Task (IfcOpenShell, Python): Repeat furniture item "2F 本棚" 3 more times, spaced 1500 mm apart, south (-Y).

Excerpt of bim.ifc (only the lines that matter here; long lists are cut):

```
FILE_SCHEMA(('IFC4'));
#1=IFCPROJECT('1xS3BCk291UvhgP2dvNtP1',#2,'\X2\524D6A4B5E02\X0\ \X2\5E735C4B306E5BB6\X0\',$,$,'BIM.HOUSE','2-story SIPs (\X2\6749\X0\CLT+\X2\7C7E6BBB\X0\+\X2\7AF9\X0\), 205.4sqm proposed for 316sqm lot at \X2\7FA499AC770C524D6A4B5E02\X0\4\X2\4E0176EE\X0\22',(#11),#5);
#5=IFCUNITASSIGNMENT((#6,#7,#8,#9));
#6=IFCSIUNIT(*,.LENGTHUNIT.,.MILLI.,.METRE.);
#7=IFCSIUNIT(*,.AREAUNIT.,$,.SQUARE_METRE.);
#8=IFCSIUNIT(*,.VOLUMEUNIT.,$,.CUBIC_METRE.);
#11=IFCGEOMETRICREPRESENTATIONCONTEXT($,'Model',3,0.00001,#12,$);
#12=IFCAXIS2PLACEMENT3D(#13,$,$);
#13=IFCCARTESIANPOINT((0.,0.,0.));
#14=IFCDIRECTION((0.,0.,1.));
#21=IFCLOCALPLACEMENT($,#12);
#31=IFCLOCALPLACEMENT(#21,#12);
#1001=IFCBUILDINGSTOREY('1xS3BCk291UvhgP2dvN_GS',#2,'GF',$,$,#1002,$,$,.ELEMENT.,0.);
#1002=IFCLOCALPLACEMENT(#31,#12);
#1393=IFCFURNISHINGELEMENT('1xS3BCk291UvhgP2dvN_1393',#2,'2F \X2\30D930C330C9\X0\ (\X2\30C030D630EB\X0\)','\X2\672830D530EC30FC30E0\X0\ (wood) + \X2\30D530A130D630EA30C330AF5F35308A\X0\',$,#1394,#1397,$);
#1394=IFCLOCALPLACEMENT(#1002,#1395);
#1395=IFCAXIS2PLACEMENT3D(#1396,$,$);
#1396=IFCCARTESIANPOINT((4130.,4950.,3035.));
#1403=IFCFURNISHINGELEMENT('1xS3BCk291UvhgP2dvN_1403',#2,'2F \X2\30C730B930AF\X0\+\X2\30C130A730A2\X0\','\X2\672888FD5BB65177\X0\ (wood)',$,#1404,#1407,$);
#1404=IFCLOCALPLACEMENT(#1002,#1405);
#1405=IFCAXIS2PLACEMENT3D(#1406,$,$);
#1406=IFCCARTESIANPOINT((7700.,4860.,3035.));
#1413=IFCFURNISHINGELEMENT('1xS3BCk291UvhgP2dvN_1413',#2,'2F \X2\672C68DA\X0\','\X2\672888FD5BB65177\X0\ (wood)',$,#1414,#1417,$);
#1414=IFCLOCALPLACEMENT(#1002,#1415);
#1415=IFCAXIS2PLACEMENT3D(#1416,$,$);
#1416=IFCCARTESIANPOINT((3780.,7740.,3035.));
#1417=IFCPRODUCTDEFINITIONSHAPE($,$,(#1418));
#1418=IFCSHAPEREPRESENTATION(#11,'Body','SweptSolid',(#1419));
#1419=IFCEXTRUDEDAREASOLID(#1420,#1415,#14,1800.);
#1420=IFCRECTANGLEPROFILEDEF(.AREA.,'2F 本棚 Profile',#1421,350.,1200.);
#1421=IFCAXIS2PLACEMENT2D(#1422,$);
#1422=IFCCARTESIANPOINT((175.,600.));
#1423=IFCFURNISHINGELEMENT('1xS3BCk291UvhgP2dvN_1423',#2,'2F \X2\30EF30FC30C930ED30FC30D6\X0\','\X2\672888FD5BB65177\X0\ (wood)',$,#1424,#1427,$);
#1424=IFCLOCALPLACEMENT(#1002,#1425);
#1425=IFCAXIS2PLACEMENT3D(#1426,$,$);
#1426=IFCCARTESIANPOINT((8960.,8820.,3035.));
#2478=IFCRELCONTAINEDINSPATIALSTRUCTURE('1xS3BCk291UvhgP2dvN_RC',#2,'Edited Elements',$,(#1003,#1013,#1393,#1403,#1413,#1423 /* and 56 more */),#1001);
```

```python
import numpy as np
import ifcopenshell
import ifcopenshell.api.geometry
import ifcopenshell.api.root
import ifcopenshell.util.element
import ifcopenshell.util.placement

model = ifcopenshell.open("bim.ifc")


def reuse_history(source, copy):
    """copy_class also copies each property set's owner history, people and application; keep the originals."""
    for rel in copy.IsDefinedBy:
        if rel.is_a("IfcRelDefinesByProperties") and (history := rel.RelatingPropertyDefinition.OwnerHistory):
            rel.RelatingPropertyDefinition.OwnerHistory = source.OwnerHistory
            ifcopenshell.util.element.remove_deep2(model, history)


source = model.by_guid("1xS3BCk291UvhgP2dvN_1413")
base = ifcopenshell.util.placement.get_local_placement(source.ObjectPlacement)
step = np.array([0.0, -1.0, 0.0]) * 1500.0

for i in range(1, 4):
    copy = ifcopenshell.api.root.copy_class(model, product=source)
    copy.Representation = ifcopenshell.util.element.copy_deep(
        model, source.Representation, exclude=["IfcGeometricRepresentationContext", "IfcRepresentationMap"]
    )
    reuse_history(source, copy)
    matrix = base.copy()
    matrix[:3, 3] += i * step
    print("added at", matrix[:3, 3].round(3) + 0.0)
    ifcopenshell.api.geometry.edit_object_placement(model, product=copy, matrix=matrix, is_si=False)

model.write("bim-out.ifc")
```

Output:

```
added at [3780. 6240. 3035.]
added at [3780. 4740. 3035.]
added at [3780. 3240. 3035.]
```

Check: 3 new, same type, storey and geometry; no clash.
